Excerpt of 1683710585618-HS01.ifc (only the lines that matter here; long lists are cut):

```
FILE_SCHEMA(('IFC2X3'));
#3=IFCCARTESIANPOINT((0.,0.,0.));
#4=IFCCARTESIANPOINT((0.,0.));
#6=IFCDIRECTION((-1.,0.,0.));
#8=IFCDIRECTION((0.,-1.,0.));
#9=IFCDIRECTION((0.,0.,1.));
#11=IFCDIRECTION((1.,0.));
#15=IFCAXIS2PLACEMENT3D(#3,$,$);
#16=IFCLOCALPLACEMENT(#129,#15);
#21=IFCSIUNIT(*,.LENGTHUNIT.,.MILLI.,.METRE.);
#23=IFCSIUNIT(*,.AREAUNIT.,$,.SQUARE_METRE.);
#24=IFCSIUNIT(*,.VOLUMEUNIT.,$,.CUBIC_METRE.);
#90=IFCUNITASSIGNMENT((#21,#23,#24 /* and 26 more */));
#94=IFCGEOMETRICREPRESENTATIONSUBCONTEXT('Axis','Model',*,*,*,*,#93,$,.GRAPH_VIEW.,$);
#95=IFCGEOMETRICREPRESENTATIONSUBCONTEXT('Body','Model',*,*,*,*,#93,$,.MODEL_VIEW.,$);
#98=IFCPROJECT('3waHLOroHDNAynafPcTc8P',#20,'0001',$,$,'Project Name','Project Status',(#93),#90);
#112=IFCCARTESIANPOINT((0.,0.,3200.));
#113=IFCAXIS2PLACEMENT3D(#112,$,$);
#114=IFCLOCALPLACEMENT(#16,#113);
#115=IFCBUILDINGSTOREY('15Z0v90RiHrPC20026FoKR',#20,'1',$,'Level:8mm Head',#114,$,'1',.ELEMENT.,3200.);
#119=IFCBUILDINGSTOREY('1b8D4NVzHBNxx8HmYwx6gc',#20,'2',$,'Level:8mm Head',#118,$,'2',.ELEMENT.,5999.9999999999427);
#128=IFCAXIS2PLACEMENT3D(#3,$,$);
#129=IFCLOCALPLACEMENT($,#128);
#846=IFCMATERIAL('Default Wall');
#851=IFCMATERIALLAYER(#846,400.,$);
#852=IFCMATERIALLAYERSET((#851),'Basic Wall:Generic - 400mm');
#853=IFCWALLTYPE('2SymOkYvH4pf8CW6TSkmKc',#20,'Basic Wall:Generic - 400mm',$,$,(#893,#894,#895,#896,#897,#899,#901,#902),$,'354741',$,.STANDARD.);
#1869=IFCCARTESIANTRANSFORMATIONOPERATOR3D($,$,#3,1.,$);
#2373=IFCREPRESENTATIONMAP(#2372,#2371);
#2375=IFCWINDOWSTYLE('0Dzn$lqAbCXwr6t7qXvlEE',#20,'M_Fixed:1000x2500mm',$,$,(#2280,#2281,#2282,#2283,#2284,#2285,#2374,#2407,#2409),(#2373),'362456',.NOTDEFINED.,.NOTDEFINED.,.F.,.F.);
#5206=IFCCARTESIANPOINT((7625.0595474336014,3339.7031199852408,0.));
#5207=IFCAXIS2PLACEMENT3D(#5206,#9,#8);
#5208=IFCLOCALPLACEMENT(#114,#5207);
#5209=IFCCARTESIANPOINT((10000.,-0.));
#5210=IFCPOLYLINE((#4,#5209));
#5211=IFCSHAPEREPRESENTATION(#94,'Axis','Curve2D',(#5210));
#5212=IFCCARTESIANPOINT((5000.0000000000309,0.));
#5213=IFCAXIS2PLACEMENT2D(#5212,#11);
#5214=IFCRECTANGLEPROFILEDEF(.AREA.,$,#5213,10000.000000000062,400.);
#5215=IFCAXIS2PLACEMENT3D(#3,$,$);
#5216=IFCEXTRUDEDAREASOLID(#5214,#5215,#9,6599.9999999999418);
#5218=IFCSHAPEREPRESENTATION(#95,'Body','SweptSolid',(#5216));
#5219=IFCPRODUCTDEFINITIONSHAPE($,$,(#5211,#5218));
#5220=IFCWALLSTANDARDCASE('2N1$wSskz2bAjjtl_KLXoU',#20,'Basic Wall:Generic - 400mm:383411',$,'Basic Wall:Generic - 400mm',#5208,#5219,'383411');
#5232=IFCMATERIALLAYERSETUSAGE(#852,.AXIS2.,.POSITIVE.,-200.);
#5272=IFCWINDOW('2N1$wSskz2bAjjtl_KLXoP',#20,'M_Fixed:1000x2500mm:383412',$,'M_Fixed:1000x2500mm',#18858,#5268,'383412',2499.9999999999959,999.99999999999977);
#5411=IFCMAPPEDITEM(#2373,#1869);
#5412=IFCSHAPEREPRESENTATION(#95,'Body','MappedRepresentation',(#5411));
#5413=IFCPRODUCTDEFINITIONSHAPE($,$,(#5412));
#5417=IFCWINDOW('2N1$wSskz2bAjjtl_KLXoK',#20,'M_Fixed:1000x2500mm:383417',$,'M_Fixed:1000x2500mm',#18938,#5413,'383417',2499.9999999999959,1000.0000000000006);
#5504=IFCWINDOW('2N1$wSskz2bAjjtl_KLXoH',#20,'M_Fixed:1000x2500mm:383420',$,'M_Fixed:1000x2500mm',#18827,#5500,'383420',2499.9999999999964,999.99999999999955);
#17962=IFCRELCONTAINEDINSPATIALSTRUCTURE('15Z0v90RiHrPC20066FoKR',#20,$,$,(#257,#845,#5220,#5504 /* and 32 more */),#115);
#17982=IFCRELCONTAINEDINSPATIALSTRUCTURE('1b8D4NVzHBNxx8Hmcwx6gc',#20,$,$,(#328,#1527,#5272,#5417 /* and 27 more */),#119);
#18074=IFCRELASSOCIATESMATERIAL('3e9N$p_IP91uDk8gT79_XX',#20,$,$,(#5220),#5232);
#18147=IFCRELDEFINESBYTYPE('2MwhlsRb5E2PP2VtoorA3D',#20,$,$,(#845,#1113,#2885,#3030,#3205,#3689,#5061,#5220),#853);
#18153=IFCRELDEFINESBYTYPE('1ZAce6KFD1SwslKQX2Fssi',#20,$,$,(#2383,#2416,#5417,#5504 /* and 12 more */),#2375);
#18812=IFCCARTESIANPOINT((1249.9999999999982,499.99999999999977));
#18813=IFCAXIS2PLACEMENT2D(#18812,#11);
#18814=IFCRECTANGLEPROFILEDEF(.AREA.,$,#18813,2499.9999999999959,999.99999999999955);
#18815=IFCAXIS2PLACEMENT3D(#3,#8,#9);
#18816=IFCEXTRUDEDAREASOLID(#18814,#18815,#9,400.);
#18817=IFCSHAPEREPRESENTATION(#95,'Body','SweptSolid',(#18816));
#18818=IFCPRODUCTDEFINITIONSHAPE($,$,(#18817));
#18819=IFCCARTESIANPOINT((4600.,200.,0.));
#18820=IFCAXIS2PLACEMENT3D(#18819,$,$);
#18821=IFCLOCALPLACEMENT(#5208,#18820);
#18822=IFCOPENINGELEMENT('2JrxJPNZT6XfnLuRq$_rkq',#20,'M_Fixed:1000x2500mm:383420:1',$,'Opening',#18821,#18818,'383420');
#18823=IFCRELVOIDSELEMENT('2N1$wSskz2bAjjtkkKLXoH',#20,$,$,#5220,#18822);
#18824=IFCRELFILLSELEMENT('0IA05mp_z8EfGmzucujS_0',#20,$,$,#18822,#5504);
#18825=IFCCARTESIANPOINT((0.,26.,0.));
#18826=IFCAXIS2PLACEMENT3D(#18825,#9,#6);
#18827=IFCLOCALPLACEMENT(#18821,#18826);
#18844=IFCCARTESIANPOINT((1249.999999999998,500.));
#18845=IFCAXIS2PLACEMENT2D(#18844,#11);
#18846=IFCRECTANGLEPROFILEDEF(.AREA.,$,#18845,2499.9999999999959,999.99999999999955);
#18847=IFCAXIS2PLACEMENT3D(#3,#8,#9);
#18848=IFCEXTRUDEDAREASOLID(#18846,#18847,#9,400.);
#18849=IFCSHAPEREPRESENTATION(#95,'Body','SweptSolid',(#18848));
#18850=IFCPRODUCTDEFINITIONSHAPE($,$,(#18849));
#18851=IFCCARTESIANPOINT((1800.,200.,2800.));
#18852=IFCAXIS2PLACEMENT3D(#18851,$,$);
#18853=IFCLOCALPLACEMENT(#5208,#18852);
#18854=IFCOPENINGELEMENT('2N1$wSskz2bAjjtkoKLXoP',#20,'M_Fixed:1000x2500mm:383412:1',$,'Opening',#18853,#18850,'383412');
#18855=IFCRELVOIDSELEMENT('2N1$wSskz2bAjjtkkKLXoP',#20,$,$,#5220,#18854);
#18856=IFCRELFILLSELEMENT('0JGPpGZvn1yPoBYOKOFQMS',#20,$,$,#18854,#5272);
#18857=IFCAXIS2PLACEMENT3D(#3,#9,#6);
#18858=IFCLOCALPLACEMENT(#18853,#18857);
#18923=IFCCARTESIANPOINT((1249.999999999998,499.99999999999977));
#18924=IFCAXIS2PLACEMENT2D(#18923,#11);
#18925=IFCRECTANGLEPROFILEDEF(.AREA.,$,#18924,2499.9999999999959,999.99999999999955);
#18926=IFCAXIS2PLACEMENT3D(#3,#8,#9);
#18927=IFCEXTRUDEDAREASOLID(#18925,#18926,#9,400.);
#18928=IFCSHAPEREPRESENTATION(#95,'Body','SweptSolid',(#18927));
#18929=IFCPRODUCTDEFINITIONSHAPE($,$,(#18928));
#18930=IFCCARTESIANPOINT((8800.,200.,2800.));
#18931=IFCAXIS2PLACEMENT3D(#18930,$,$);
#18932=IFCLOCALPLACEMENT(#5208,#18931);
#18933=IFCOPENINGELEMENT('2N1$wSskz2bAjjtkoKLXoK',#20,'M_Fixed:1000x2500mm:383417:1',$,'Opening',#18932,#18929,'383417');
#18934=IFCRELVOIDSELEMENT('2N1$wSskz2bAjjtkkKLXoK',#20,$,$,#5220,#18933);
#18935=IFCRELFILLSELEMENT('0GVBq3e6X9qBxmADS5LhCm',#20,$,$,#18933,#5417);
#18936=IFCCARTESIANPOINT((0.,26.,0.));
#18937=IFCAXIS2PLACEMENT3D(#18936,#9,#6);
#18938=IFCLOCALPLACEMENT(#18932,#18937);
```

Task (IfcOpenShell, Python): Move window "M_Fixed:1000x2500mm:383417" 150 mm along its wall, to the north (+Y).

```python
import ifcopenshell
import ifcopenshell.api.geometry
import ifcopenshell.util.placement

model = ifcopenshell.open("1683710585618-HS01.ifc")

window = model.by_guid("2N1$wSskz2bAjjtl_KLXoK")
opening = window.FillsVoids[0].RelatingOpeningElement
wall = opening.VoidsElements[0].RelatingBuildingElement

wall_matrix = ifcopenshell.util.placement.get_local_placement(wall.ObjectPlacement)
shift = wall_matrix[:3, 0] * -150.0
before = ifcopenshell.util.placement.get_local_placement(window.ObjectPlacement)[:3, 3].copy()

# The window is placed relative to its opening, so it follows when the opening moves.
matrix = ifcopenshell.util.placement.get_local_placement(opening.ObjectPlacement)
matrix[:3, 3] += shift
ifcopenshell.api.geometry.edit_object_placement(
    model, product=opening, matrix=matrix, is_si=False, should_transform_children=True
)

after = ifcopenshell.util.placement.get_local_placement(window.ObjectPlacement)[:3, 3]
print("window moved by", (after - before).round(3) + 0.0)

model.write("1683710585618-HS01_v2.ifc")
```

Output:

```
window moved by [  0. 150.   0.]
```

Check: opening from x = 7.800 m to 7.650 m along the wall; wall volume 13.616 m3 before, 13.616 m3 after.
